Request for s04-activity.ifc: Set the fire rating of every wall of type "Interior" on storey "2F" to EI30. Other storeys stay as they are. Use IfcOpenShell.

First a look at what the model holds.

```python
import ifcopenshell
import ifcopenshell.util.element

model = ifcopenshell.open("s04-activity.ifc")
print(model.schema)
storey = next(s for s in model.by_type("IfcBuildingStorey") if s.Name == "2F")
walls = [e for e in ifcopenshell.util.element.get_decomposition(storey) if e.is_a("IfcWall")]
seen = {}
for e in walls:
    element_type = ifcopenshell.util.element.get_type(e)
    key = (element_type.Name if element_type != e and element_type else None, ifcopenshell.util.element.get_pset(e, "Pset_WallCommon", "FireRating"))
    seen[key] = seen.get(key, 0) + 1
for (name, value), count in sorted(seen.items(), key=str):
    print(count, "x", name, "|", value)
```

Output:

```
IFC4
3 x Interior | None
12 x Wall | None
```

```python
import ifcopenshell
import ifcopenshell.api.pset
import ifcopenshell.util.element

model = ifcopenshell.open("s04-activity.ifc")

storey = next(s for s in model.by_type("IfcBuildingStorey") if s.Name == "2F")
walls = [e for e in ifcopenshell.util.element.get_decomposition(storey) if e.is_a("IfcWall")]

count = 0
for e in walls:
    element_type = ifcopenshell.util.element.get_type(e)
    if element_type in (None, e) or element_type.Name != "Interior":
        continue
    # add_pset returns the element's existing set when there is one.
    pset = ifcopenshell.api.pset.add_pset(model, product=e, name="Pset_WallCommon")
    ifcopenshell.api.pset.edit_pset(model, pset=pset, properties={"FireRating": "EI30"})
    count += 1

print(count, "walls updated")

model.write("s04-activity_updated.ifc")
```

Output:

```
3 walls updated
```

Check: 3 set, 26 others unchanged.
